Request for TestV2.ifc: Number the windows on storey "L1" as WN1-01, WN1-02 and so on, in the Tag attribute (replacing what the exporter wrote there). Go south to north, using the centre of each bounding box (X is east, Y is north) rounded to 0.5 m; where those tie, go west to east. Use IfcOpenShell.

First a look at what the model holds.

```python
import ifcopenshell
import ifcopenshell.util.element
import ifcopenshell.util.placement

model = ifcopenshell.open("TestV2.ifc")
print(model.schema)
storey = next(s for s in model.by_type("IfcBuildingStorey") if s.Name == "L1")
windows = [e for e in ifcopenshell.util.element.get_decomposition(storey) if e.is_a("IfcWindow")]
for e in sorted(windows, key=lambda e: e.id()):
    origin = ifcopenshell.util.placement.get_local_placement(e.ObjectPlacement)[:3, 3]
    print(e.id(), e.Tag, e.Name, origin.round(2) + 0.0, sep=" | ")
```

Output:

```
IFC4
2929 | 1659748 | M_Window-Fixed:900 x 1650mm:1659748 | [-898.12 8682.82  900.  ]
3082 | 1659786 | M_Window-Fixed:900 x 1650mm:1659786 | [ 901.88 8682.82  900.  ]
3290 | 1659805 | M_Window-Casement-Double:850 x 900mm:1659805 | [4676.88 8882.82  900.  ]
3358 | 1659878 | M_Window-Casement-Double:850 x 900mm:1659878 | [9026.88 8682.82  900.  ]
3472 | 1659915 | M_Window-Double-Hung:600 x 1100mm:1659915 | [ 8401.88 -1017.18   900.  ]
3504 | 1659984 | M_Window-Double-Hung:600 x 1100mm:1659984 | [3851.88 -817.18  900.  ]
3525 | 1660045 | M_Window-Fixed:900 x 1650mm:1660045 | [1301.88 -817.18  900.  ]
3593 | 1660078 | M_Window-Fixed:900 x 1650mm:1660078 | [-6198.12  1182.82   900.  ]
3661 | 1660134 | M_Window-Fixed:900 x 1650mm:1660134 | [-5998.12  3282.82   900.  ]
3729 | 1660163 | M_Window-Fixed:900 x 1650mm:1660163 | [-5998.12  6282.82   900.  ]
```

```python
import ifcopenshell
import ifcopenshell.geom
import ifcopenshell.util.element
import ifcopenshell.util.shape

model = ifcopenshell.open("TestV2.ifc")
settings = ifcopenshell.geom.settings()
settings.set("use-world-coords", True)


def centre(element):
    shape = ifcopenshell.geom.create_shape(settings, element)
    return ifcopenshell.util.shape.get_bbox_centroid(shape.geometry)


storey = next(s for s in model.by_type("IfcBuildingStorey") if s.Name == "L1")
windows = [e for e in ifcopenshell.util.element.get_decomposition(storey) if e.is_a("IfcWindow")]

# Insertion points can sit at a corner or the storey origin, so sort by the geometry (in metres).
centres = {e: centre(e) for e in windows}
windows.sort(key=lambda e: (round(centres[e][1] / 0.5), centres[e][0]))

for i, e in enumerate(windows, start=1):
    number = f"WN1-{i:02d}"
    e.Tag = number
    print(e.id(), number)

model.write("TestV2_rev.ifc")
```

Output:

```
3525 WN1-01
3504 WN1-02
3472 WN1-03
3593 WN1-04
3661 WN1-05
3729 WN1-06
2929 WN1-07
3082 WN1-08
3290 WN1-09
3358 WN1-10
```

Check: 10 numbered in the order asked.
